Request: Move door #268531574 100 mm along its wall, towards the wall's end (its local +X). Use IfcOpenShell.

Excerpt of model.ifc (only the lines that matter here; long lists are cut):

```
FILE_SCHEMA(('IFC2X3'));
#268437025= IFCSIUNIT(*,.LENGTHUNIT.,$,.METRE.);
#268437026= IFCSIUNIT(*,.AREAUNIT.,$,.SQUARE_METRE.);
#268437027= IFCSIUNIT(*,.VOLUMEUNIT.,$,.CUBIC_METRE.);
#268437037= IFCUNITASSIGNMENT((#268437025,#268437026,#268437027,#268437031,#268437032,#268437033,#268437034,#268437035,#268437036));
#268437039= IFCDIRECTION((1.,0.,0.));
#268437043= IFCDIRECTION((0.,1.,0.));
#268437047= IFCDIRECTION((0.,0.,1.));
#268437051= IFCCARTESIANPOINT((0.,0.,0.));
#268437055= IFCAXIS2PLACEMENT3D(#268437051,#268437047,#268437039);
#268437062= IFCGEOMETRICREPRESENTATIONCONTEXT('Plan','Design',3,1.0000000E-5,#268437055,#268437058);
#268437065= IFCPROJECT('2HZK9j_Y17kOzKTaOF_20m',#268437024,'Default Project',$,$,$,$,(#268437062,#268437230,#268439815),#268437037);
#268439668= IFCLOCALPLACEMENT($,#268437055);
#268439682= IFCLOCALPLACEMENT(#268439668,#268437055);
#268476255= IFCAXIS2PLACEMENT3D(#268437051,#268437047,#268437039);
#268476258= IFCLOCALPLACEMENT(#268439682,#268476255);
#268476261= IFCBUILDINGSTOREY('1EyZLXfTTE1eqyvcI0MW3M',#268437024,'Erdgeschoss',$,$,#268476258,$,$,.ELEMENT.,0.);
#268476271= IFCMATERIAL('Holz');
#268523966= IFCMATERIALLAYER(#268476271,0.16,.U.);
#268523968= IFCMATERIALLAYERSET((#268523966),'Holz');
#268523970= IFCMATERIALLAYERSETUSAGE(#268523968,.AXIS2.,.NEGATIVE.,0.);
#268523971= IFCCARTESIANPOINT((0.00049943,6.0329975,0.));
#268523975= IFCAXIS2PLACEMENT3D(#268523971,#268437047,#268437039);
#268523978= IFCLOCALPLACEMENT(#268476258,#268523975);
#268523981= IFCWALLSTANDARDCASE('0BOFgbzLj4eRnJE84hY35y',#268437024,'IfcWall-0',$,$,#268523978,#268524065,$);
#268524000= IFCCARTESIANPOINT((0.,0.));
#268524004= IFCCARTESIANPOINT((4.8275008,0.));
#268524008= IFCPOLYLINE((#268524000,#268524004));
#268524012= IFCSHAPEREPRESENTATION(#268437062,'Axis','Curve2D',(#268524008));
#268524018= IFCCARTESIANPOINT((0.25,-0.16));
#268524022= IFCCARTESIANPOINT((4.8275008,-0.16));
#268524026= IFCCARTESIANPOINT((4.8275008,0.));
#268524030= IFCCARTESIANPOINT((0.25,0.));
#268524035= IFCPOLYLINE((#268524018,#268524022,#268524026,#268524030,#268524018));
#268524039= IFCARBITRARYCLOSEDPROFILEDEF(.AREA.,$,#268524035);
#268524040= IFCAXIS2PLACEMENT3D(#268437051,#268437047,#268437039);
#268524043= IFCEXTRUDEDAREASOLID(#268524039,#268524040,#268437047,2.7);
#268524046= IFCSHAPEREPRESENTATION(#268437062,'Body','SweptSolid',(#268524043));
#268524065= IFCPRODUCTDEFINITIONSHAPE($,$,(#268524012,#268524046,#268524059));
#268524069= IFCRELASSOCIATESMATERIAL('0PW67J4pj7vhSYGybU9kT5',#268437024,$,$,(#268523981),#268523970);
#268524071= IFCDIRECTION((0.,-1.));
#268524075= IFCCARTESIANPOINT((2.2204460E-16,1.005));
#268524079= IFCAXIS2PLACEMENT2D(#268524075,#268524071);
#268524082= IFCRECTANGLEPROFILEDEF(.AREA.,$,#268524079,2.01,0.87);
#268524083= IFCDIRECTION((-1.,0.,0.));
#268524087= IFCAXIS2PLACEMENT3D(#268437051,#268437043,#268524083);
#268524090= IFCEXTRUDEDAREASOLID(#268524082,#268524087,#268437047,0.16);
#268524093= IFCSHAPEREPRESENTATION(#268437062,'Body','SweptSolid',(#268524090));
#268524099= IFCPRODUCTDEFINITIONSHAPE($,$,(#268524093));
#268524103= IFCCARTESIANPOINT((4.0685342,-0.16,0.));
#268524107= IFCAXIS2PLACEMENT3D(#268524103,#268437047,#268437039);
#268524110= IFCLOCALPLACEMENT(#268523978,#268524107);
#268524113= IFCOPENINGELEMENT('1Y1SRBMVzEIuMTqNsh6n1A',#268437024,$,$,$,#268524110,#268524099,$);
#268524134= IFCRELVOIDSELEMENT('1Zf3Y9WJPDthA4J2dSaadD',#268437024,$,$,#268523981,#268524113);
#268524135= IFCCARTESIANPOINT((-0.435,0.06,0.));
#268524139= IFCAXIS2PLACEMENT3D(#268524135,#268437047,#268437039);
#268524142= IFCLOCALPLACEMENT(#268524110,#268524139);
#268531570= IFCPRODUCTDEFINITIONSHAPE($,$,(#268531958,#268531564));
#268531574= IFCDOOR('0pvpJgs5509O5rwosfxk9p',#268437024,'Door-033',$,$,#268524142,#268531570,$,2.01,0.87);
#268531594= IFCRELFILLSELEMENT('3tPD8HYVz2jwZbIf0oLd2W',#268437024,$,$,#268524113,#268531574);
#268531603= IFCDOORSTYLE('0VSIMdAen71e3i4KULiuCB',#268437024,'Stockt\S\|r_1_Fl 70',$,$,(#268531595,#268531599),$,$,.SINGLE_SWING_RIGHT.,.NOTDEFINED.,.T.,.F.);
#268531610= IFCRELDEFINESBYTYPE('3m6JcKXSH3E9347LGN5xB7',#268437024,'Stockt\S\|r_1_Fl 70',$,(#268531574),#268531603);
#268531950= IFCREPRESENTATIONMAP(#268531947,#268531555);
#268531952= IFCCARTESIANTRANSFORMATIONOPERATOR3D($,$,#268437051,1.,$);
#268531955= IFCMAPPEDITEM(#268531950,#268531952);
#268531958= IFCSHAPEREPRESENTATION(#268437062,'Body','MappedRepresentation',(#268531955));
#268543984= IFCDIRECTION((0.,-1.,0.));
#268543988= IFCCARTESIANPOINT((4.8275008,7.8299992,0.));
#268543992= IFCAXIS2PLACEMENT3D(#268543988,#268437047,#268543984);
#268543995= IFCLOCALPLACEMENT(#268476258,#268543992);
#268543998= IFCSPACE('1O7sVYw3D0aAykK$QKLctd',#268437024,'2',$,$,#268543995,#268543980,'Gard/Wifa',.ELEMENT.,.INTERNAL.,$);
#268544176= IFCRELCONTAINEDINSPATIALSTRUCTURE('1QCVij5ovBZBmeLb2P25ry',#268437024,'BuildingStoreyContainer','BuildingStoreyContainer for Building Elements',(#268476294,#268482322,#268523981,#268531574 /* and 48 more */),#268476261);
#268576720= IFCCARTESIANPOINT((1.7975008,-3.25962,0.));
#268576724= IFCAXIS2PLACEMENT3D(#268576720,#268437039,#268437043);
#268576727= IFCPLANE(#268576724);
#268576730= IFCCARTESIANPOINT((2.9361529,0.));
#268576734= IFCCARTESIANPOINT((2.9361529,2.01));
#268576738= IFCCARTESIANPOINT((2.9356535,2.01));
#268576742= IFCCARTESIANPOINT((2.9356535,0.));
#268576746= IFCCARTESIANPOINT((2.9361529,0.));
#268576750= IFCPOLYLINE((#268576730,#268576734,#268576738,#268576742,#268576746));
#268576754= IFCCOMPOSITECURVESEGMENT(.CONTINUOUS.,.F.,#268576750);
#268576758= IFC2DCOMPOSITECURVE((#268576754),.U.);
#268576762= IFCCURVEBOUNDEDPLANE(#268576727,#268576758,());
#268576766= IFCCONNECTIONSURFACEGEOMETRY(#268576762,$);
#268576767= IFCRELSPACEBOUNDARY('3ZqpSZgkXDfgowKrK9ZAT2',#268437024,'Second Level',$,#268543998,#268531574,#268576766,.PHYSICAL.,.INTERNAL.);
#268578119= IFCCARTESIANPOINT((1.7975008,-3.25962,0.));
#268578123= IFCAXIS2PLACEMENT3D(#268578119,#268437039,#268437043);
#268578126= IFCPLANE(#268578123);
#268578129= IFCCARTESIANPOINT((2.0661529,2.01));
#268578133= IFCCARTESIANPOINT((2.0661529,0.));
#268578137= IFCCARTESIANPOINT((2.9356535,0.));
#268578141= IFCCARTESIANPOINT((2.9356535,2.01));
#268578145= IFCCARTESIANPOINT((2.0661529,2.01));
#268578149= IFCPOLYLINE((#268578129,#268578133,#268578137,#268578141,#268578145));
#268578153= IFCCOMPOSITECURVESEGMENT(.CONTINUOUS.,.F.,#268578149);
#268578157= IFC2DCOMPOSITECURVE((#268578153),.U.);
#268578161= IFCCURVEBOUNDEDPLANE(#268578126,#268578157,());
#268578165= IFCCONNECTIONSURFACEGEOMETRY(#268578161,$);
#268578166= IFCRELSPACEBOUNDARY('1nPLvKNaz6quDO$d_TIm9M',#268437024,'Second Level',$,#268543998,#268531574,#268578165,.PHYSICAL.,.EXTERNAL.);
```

```python
import numpy as np
import ifcopenshell
import ifcopenshell.api.geometry
import ifcopenshell.util.placement
import ifcopenshell.util.unit

model = ifcopenshell.open("model.ifc")
unit_scale = ifcopenshell.util.unit.calculate_unit_scale(model)

door = model.by_guid("0pvpJgs5509O5rwosfxk9p")
opening = door.FillsVoids[0].RelatingOpeningElement
wall = opening.VoidsElements[0].RelatingBuildingElement

wall_matrix = ifcopenshell.util.placement.get_local_placement(wall.ObjectPlacement)
shift = wall_matrix[:3, 0] * 0.1 / unit_scale
before = ifcopenshell.util.placement.get_local_placement(door.ObjectPlacement)[:3, 3].copy()

# The door is placed relative to its opening, so it follows when the opening moves.
matrix = ifcopenshell.util.placement.get_local_placement(opening.ObjectPlacement)
matrix[:3, 3] += shift
ifcopenshell.api.geometry.edit_object_placement(
    model, product=opening, matrix=matrix, is_si=False, should_transform_children=True
)

# Space boundary surfaces are stored in each space's coordinates; move them too.
for rel in door.ProvidesBoundaries:
    if not rel.ConnectionGeometry:
        continue
    surface = rel.ConnectionGeometry.SurfaceOnRelatingElement.BasisSurface
    space_matrix = ifcopenshell.util.placement.get_local_placement(rel.RelatingSpace.ObjectPlacement)
    point = np.array(surface.Position.Location.Coordinates) + space_matrix[:3, :3].T @ shift
    surface.Position = model.createIfcAxis2Placement3D(
        model.createIfcCartesianPoint(point.tolist()), surface.Position.Axis, surface.Position.RefDirection
    )

after = ifcopenshell.util.placement.get_local_placement(door.ObjectPlacement)[:3, 3]
print("door moved by", (after - before).round(3) + 0.0)

model.write("model-out.ifc")
```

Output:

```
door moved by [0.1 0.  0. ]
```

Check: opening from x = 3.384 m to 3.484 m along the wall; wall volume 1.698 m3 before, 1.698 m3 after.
